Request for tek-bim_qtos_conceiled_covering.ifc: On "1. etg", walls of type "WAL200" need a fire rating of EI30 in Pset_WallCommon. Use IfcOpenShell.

First a look at what the model holds.

```python
import ifcopenshell
import ifcopenshell.util.element

model = ifcopenshell.open("tek-bim_qtos_conceiled_covering.ifc")
print(model.schema)
storey = next(s for s in model.by_type("IfcBuildingStorey") if s.Name == "1. etg")
walls = [e for e in ifcopenshell.util.element.get_decomposition(storey) if e.is_a("IfcWall")]
seen = {}
for e in walls:
    element_type = ifcopenshell.util.element.get_type(e)
    key = (element_type.Name if element_type != e and element_type else None, ifcopenshell.util.element.get_pset(e, "Pset_WallCommon", "FireRating"))
    seen[key] = seen.get(key, 0) + 1
for (name, value), count in sorted(seen.items(), key=str):
    print(count, "x", name, "|", value)
```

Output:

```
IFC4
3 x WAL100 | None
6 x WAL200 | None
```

```python
import ifcopenshell
import ifcopenshell.api.pset
import ifcopenshell.util.element

model = ifcopenshell.open("tek-bim_qtos_conceiled_covering.ifc")

storey = next(s for s in model.by_type("IfcBuildingStorey") if s.Name == "1. etg")
walls = [e for e in ifcopenshell.util.element.get_decomposition(storey) if e.is_a("IfcWall")]

count = 0
for e in walls:
    element_type = ifcopenshell.util.element.get_type(e)
    if element_type in (None, e) or element_type.Name != "WAL200":
        continue
    # add_pset returns the element's existing set when there is one.
    pset = ifcopenshell.api.pset.add_pset(model, product=e, name="Pset_WallCommon")
    ifcopenshell.api.pset.edit_pset(model, pset=pset, properties={"FireRating": "EI30"})
    count += 1

print(count, "walls updated")

model.write("tek-bim_qtos_conceiled_covering_v2.ifc")
```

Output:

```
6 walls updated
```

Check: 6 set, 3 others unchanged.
